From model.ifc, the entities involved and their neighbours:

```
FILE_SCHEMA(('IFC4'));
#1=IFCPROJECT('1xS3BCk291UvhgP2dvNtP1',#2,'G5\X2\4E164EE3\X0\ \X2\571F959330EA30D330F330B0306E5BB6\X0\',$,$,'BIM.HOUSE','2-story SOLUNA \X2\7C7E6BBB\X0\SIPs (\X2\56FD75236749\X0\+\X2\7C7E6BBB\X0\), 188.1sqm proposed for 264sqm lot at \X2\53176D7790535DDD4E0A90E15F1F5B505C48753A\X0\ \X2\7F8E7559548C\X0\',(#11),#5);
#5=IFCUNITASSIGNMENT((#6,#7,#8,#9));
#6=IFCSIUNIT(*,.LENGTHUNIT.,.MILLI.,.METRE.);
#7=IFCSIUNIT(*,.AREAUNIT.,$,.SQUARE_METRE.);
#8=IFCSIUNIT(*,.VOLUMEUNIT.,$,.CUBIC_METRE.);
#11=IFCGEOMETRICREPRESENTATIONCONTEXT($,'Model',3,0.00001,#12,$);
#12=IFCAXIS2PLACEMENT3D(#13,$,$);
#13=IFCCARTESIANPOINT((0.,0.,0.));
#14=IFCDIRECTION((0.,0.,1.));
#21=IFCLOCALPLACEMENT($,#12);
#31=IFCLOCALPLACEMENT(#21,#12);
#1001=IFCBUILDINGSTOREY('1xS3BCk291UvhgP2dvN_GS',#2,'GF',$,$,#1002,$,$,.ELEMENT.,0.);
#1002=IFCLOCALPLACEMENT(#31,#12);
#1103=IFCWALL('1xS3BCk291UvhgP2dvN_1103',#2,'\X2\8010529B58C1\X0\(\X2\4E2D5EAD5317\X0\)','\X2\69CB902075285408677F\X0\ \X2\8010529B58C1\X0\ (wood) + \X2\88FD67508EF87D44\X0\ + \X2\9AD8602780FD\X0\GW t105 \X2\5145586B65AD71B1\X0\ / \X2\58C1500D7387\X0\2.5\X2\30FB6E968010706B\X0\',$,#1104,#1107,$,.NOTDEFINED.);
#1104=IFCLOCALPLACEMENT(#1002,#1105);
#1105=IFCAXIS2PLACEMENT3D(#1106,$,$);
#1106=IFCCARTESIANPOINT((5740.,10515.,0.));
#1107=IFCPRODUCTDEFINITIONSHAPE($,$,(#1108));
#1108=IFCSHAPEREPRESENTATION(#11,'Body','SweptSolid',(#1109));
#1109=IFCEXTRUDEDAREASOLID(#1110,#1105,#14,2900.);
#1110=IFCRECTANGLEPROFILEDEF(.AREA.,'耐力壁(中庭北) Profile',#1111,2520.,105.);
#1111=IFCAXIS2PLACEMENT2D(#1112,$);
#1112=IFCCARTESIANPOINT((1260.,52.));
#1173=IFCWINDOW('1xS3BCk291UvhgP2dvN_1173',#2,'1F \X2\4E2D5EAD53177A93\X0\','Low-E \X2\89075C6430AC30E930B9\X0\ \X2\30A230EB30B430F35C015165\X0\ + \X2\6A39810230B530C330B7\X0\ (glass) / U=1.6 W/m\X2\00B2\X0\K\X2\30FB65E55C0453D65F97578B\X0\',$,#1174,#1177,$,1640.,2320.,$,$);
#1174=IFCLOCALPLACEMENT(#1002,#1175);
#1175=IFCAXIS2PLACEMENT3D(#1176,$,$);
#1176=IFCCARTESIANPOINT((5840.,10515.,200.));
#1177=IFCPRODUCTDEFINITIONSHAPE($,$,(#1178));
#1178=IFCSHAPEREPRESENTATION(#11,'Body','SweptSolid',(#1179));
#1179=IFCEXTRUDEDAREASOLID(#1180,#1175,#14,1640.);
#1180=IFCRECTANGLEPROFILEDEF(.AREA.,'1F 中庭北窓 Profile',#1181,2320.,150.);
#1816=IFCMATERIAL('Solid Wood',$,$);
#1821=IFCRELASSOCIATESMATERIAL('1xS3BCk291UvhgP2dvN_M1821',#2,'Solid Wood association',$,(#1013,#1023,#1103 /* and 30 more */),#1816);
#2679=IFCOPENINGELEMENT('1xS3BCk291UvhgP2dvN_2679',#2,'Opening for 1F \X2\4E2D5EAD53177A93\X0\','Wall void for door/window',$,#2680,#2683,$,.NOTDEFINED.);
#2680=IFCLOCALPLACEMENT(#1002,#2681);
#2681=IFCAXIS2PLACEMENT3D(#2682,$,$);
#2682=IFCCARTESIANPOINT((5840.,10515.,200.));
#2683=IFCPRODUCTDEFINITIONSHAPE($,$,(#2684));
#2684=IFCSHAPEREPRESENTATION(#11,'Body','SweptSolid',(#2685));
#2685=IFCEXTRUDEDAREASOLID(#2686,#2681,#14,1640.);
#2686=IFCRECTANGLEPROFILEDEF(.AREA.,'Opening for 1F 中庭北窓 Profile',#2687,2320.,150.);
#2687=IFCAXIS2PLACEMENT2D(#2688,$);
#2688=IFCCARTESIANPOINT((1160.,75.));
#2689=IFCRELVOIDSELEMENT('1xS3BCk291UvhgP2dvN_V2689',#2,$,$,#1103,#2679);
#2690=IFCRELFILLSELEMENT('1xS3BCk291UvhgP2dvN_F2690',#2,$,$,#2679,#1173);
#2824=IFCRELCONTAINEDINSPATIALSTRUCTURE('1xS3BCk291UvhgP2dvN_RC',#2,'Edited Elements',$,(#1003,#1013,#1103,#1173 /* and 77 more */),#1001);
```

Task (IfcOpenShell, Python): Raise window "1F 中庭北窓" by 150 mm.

```python
import numpy as np
import ifcopenshell
import ifcopenshell.api.geometry
import ifcopenshell.util.placement
import ifcopenshell.util.unit

model = ifcopenshell.open("model.ifc")
unit_scale = ifcopenshell.util.unit.calculate_unit_scale(model)

window = model.by_guid("1xS3BCk291UvhgP2dvN_1173")
opening = window.FillsVoids[0].RelatingOpeningElement
dz = 0.15 / unit_scale

shift = np.array([0.0, 0.0, dz])
# The window is not placed relative to its opening, so move both.
for product in (opening, window):
    matrix = ifcopenshell.util.placement.get_local_placement(product.ObjectPlacement)
    matrix[:3, 3] += shift
    ifcopenshell.api.geometry.edit_object_placement(model, product=product, matrix=matrix, is_si=False)

print(f"moved by {dz * unit_scale:+.3f} m")

model.write("model_updated.ifc")
```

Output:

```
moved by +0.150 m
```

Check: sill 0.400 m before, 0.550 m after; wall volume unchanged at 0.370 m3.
